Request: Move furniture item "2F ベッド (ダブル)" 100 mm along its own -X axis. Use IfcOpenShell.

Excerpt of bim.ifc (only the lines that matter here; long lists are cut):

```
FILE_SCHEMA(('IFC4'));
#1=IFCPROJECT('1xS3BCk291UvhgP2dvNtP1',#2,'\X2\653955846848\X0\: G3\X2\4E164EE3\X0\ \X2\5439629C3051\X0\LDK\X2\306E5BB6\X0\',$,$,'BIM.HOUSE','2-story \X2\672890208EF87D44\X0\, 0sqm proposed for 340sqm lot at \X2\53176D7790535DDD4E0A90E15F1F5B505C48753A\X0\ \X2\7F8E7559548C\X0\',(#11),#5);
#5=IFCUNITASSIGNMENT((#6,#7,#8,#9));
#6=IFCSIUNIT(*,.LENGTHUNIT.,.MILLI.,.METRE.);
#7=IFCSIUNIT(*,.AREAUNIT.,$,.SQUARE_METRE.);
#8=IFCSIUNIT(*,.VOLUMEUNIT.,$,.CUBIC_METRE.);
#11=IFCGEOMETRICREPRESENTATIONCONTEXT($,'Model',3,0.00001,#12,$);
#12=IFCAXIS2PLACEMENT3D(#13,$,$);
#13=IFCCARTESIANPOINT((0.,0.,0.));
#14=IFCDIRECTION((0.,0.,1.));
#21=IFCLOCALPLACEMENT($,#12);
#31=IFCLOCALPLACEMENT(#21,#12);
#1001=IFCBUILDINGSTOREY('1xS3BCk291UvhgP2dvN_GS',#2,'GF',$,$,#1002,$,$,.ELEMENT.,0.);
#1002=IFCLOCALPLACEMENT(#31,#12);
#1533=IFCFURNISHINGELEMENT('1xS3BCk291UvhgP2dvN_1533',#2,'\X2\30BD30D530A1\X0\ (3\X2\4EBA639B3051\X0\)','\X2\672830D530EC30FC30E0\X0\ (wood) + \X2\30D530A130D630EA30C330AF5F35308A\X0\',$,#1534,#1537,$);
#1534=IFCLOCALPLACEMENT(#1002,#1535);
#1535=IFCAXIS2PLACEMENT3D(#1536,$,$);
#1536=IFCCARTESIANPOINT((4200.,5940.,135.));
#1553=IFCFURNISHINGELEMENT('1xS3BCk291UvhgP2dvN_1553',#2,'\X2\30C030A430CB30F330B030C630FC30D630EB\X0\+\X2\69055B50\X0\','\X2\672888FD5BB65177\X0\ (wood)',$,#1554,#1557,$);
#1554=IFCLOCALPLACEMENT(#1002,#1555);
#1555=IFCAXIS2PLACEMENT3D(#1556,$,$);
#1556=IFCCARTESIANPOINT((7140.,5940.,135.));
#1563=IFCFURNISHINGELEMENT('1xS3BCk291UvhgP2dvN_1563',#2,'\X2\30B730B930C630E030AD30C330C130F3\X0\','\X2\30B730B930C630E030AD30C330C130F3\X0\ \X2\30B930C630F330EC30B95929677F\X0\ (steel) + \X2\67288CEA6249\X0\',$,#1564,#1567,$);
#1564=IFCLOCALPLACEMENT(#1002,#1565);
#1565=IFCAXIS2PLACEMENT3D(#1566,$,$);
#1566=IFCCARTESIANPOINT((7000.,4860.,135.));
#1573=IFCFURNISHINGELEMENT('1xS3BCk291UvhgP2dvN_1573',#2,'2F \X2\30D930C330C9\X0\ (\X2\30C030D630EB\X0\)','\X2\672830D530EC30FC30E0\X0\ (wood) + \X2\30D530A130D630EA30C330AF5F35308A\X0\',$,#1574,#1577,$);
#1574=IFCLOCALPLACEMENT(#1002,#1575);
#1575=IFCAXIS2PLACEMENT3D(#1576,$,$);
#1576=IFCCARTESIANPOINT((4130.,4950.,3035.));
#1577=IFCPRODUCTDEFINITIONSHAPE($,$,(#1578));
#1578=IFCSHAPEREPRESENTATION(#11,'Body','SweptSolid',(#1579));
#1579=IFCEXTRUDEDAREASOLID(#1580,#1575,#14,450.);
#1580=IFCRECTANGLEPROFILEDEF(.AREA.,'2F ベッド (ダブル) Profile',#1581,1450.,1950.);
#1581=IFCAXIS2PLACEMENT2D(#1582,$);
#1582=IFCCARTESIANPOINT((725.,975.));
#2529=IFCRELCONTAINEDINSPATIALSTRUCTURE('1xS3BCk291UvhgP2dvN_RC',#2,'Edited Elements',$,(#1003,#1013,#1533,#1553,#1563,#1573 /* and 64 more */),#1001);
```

```python
import ifcopenshell
import ifcopenshell.api.geometry
import ifcopenshell.util.placement
import ifcopenshell.util.unit

model = ifcopenshell.open("bim.ifc")
unit_scale = ifcopenshell.util.unit.calculate_unit_scale(model)

item = model.by_guid("1xS3BCk291UvhgP2dvN_1573")
matrix = ifcopenshell.util.placement.get_local_placement(item.ObjectPlacement)
matrix[:3, 3] -= matrix[:3, 0] * 0.1 / unit_scale
ifcopenshell.api.geometry.edit_object_placement(model, product=item, matrix=matrix, is_si=False)

print(ifcopenshell.util.placement.get_local_placement(item.ObjectPlacement).round(3) + 0.0)

model.write("bim_updated.ifc")
```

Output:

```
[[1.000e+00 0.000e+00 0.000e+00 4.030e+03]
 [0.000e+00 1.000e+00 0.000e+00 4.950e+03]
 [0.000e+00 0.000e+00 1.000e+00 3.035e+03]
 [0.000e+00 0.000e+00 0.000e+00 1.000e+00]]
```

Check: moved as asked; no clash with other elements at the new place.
